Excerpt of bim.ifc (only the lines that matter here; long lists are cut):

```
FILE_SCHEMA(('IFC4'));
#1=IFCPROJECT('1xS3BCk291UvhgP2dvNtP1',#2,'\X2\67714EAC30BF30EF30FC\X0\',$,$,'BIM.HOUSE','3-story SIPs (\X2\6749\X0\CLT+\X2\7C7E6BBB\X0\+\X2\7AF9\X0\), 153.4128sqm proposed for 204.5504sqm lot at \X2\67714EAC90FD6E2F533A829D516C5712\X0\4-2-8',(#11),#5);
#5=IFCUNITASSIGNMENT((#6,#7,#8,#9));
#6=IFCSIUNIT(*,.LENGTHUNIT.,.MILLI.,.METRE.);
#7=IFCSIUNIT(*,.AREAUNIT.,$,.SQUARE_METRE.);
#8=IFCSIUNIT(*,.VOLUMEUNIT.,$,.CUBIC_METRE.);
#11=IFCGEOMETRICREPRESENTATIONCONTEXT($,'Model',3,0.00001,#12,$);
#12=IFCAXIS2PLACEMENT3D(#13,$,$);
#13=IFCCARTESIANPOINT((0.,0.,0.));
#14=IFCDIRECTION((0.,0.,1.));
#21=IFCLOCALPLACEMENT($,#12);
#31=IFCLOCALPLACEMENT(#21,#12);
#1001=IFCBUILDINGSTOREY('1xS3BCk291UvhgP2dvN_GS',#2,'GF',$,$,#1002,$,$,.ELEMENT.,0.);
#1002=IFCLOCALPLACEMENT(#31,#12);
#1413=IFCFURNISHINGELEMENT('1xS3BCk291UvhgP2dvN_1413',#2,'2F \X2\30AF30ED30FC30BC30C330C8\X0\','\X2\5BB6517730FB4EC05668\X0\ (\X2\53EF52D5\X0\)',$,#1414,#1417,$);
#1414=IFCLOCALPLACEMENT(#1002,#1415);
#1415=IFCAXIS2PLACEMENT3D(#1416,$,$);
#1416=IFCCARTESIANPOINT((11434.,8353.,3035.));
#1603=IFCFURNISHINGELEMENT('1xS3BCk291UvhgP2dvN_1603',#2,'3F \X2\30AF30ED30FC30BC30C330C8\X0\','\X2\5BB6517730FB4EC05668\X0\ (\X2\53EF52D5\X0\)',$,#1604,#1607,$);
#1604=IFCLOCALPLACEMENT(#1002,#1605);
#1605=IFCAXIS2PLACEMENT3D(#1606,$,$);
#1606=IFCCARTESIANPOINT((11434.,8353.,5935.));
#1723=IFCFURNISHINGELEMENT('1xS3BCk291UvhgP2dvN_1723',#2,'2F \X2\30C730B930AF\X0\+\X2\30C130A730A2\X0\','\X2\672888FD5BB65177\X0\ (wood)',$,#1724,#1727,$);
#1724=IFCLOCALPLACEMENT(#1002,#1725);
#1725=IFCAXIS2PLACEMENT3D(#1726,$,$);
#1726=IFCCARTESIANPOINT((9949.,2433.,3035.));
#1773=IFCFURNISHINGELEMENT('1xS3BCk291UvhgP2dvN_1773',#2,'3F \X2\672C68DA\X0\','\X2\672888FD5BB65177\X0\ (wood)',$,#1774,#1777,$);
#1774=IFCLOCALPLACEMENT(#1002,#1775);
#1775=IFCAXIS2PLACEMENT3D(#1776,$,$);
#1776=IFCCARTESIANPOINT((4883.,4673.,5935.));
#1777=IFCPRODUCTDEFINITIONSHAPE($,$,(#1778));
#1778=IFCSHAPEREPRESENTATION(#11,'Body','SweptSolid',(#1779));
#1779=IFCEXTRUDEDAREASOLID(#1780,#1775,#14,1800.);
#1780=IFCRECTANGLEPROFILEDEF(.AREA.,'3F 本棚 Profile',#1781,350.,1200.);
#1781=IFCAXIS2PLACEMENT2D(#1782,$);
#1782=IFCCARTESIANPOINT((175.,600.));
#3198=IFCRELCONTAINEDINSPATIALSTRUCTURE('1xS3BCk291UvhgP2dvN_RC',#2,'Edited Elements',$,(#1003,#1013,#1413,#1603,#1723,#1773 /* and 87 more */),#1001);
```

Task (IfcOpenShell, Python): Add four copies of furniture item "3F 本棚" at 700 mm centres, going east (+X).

```python
import numpy as np
import ifcopenshell
import ifcopenshell.api.geometry
import ifcopenshell.api.root
import ifcopenshell.util.element
import ifcopenshell.util.placement

model = ifcopenshell.open("bim.ifc")


def reuse_history(source, copy):
    """copy_class also copies each property set's owner history, people and application; keep the originals."""
    for rel in copy.IsDefinedBy:
        if rel.is_a("IfcRelDefinesByProperties") and (history := rel.RelatingPropertyDefinition.OwnerHistory):
            rel.RelatingPropertyDefinition.OwnerHistory = source.OwnerHistory
            ifcopenshell.util.element.remove_deep2(model, history)


source = model.by_guid("1xS3BCk291UvhgP2dvN_1773")
base = ifcopenshell.util.placement.get_local_placement(source.ObjectPlacement)
step = np.array([1.0, 0.0, 0.0]) * 700.0

for i in range(1, 5):
    copy = ifcopenshell.api.root.copy_class(model, product=source)
    copy.Representation = ifcopenshell.util.element.copy_deep(
        model, source.Representation, exclude=["IfcGeometricRepresentationContext", "IfcRepresentationMap"]
    )
    reuse_history(source, copy)
    matrix = base.copy()
    matrix[:3, 3] += i * step
    print("added at", matrix[:3, 3].round(3) + 0.0)
    ifcopenshell.api.geometry.edit_object_placement(model, product=copy, matrix=matrix, is_si=False)

model.write("bim_rev.ifc")
```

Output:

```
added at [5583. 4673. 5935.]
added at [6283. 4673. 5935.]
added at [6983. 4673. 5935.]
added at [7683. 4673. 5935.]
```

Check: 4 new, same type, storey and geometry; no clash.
